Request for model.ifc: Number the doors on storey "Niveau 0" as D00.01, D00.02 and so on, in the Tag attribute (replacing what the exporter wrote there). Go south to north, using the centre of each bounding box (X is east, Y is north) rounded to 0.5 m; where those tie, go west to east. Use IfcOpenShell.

First a look at what the model holds.

```python
import ifcopenshell
import ifcopenshell.util.element
import ifcopenshell.util.placement

model = ifcopenshell.open("model.ifc")
print(model.schema)
storey = next(s for s in model.by_type("IfcBuildingStorey") if s.Name == "Niveau 0")
doors = [e for e in ifcopenshell.util.element.get_decomposition(storey) if e.is_a("IfcDoor")]
for e in sorted(doors, key=lambda e: e.id()):
    origin = ifcopenshell.util.placement.get_local_placement(e.ObjectPlacement)[:3, 3]
    print(e.id(), e.Tag, e.Name, origin.round(2) + 0.0, sep=" | ")
```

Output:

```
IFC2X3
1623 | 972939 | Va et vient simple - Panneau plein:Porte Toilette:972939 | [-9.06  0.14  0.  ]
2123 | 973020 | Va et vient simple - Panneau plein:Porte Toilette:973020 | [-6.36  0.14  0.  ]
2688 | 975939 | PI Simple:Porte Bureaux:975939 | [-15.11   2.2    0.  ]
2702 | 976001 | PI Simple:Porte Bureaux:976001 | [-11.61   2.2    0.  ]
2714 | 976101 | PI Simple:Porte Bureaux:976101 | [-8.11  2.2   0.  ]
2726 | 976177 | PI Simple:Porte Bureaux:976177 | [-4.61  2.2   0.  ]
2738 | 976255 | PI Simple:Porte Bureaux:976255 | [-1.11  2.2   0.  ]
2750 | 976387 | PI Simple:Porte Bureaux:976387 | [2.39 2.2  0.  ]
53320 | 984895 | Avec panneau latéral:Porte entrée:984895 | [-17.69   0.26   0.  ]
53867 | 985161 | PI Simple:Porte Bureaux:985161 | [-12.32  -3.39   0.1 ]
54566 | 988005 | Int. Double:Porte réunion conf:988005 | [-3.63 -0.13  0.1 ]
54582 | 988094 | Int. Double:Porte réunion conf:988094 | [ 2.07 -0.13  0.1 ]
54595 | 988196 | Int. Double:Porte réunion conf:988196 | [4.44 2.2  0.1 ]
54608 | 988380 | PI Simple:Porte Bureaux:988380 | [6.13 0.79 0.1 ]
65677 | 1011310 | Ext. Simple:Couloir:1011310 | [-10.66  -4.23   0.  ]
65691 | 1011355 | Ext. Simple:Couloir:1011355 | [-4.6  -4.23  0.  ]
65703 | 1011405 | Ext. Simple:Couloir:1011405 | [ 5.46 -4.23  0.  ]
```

```python
import ifcopenshell
import ifcopenshell.geom
import ifcopenshell.util.element
import ifcopenshell.util.shape

model = ifcopenshell.open("model.ifc")
settings = ifcopenshell.geom.settings()
settings.set("use-world-coords", True)


def centre(element):
    shape = ifcopenshell.geom.create_shape(settings, element)
    return ifcopenshell.util.shape.get_bbox_centroid(shape.geometry)


storey = next(s for s in model.by_type("IfcBuildingStorey") if s.Name == "Niveau 0")
doors = [e for e in ifcopenshell.util.element.get_decomposition(storey) if e.is_a("IfcDoor")]

# Insertion points can sit at a corner or the storey origin, so sort by the geometry (in metres).
centres = {e: centre(e) for e in doors}
doors.sort(key=lambda e: (round(centres[e][1] / 0.5), centres[e][0]))

for i, e in enumerate(doors, start=1):
    number = f"D00.{i:02d}"
    e.Tag = number
    print(e.id(), number)

model.write("model_edited.ifc")
```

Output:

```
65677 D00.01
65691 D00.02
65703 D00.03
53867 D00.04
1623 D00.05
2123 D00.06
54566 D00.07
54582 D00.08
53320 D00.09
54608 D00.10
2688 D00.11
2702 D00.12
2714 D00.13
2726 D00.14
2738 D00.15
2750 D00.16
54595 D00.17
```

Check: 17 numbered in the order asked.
